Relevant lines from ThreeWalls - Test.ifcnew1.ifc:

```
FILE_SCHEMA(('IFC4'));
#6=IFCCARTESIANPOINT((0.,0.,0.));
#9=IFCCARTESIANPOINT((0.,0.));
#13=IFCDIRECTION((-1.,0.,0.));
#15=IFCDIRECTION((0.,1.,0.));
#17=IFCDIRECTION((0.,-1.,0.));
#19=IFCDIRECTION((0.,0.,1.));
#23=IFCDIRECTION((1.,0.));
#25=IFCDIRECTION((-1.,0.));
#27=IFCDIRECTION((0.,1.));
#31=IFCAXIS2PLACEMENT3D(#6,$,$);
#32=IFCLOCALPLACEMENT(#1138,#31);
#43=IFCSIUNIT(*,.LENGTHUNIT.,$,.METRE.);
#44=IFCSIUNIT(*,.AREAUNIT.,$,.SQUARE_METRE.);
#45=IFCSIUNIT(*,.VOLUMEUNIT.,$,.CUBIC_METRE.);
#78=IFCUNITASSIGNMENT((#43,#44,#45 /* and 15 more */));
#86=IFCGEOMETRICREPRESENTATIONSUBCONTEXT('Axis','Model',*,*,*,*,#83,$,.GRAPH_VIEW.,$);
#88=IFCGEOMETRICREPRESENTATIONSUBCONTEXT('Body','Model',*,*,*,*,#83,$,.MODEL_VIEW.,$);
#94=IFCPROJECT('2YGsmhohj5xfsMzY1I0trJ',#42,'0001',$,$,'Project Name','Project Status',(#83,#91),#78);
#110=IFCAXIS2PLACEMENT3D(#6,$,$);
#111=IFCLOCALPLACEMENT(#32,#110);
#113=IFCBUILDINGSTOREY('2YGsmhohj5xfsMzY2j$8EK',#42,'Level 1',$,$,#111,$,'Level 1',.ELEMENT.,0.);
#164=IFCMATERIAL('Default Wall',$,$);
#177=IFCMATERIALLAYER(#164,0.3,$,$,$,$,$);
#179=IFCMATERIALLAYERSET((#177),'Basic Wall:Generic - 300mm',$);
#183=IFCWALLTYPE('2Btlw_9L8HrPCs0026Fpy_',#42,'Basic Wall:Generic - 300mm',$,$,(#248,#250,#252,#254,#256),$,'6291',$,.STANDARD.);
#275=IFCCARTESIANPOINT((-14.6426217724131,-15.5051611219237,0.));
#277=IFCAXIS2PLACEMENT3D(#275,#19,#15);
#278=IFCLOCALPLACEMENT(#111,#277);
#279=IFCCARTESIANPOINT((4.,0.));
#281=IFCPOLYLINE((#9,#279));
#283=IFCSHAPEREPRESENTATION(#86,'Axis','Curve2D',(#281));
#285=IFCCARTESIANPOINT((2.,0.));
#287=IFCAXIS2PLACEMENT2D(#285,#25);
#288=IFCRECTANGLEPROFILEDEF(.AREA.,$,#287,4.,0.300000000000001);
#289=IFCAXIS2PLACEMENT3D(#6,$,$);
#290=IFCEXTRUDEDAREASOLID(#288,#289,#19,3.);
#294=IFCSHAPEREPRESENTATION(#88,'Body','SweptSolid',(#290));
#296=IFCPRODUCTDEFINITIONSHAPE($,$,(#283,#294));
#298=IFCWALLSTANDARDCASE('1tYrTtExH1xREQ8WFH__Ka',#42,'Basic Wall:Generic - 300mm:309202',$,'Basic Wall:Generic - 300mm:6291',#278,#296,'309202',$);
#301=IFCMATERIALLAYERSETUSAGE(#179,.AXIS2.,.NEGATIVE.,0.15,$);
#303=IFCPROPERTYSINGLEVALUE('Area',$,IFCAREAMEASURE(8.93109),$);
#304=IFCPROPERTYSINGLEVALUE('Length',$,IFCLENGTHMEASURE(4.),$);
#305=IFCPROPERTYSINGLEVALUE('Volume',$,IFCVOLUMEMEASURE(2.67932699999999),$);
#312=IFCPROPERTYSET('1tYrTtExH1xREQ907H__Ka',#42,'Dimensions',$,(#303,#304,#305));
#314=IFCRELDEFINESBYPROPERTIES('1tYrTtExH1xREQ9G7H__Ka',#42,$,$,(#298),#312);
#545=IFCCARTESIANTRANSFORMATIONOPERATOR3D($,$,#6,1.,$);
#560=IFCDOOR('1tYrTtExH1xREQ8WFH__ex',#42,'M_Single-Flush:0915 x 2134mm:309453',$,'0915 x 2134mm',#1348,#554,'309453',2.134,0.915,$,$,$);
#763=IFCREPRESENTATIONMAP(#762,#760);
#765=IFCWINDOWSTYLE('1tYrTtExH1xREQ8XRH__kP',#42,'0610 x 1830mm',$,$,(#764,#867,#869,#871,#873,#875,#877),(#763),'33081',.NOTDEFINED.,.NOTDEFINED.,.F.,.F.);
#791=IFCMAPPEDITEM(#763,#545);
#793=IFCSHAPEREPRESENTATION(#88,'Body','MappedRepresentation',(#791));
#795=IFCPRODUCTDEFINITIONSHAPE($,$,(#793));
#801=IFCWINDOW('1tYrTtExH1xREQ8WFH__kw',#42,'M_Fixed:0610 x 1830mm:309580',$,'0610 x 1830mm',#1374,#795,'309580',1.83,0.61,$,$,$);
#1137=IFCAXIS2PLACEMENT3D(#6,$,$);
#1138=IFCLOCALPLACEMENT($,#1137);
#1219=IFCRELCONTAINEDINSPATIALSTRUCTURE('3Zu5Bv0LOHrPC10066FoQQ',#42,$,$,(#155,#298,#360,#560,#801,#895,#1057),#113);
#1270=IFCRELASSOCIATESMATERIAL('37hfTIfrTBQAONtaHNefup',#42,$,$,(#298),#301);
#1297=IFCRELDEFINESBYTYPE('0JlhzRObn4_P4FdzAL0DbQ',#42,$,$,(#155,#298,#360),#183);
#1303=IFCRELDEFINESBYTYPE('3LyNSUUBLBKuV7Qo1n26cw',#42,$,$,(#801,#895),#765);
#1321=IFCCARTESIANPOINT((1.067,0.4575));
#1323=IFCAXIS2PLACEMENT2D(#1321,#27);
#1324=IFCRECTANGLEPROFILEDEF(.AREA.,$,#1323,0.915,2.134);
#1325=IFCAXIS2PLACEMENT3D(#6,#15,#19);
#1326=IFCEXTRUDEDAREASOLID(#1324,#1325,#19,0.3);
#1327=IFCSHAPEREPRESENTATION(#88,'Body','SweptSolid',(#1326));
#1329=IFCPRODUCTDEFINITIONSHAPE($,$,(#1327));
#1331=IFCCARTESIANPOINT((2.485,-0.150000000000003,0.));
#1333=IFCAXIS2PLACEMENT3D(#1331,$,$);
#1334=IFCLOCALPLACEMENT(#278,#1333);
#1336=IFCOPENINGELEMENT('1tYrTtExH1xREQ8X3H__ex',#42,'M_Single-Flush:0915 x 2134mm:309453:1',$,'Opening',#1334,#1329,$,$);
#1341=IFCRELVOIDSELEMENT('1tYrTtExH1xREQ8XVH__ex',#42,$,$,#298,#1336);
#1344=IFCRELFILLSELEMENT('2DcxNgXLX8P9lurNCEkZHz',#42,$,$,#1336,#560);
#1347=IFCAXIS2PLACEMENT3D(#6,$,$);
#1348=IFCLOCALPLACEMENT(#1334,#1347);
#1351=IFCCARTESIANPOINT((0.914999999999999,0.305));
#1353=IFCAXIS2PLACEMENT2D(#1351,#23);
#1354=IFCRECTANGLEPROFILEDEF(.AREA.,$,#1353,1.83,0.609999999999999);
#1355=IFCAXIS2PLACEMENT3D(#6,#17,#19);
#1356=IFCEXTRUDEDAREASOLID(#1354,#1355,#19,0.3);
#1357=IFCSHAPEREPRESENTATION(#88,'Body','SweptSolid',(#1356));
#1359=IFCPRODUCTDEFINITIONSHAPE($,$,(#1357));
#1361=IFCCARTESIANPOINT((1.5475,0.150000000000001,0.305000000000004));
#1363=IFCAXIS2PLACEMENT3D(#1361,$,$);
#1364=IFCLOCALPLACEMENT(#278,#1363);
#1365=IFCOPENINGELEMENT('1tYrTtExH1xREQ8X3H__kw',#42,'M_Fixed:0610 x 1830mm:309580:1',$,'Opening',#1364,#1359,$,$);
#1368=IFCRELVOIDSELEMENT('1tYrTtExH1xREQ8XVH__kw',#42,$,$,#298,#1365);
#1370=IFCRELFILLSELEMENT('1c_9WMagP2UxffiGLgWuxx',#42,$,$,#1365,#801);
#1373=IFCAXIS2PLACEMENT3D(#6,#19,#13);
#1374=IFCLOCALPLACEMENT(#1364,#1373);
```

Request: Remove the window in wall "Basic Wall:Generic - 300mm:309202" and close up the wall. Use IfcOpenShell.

```python
import ifcopenshell
import ifcopenshell.api.feature
import ifcopenshell.api.pset
import ifcopenshell.api.root
import ifcopenshell.geom
import ifcopenshell.util.element
import ifcopenshell.util.shape
import ifcopenshell.util.unit

model = ifcopenshell.open("ThreeWalls - Test.ifcnew1.ifc")
area_scale = ifcopenshell.util.unit.calculate_unit_scale(model, "AREAUNIT")
volume_scale = ifcopenshell.util.unit.calculate_unit_scale(model, "VOLUMEUNIT")
settings = ifcopenshell.geom.settings()


def volume(element):
    """Net volume in cubic metres, openings subtracted."""
    shape = ifcopenshell.geom.create_shape(settings, element)
    return ifcopenshell.util.shape.get_volume(shape.geometry)


window = model.by_guid("1tYrTtExH1xREQ8WFH__kw")
opening = window.FillsVoids[0].RelatingOpeningElement
wall = opening.VoidsElements[0].RelatingBuildingElement
before = volume(wall)

ifcopenshell.api.root.remove_product(model, product=window)
ifcopenshell.api.feature.remove_feature(model, feature=opening)

after = volume(wall)
thickness = 0.3  # wall thickness in metres

# Update the wall's stored quantities.
pset = model.by_id(ifcopenshell.util.element.get_pset(wall, "Dimensions", should_inherit=False)["id"])
ifcopenshell.api.pset.edit_pset(model, pset=pset, properties={
    "Area": model.create_entity("IfcAreaMeasure", after / thickness / area_scale),
    "Volume": model.create_entity("IfcVolumeMeasure", after / volume_scale),
})

print(f"wall volume {before:.3f} -> {after:.3f} m3")

model.write("ThreeWalls - Test.ifcnew1_updated.ifc")
```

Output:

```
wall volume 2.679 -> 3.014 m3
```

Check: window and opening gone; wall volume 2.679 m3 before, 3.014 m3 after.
